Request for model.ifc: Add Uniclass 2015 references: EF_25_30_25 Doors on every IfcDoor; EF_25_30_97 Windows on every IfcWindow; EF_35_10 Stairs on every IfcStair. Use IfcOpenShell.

First a look at what the model holds.

```python
import ifcopenshell

model = ifcopenshell.open("model.ifc")
print(model.schema)
print("classifications:", [c.Name for c in model.by_type("IfcClassification")])
for ifc_class in ("IfcDoor", "IfcRoof", "IfcStair", "IfcWall", "IfcWindow"):
    print(ifc_class, len(model.by_type(ifc_class)))
```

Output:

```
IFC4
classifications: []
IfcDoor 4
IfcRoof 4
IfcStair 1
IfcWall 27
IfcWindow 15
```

```python
import ifcopenshell
import ifcopenshell.api.classification

model = ifcopenshell.open("model.ifc")

system = ifcopenshell.api.classification.add_classification(model, classification="Uniclass 2015")

codes = {
    "IfcDoor": ("EF_25_30_25", "Doors"),
    "IfcWindow": ("EF_25_30_97", "Windows"),
    "IfcStair": ("EF_35_10", "Stairs"),
}
for ifc_class, (code, name) in codes.items():
    products = model.by_type(ifc_class)
    ifcopenshell.api.classification.add_reference(
        model, products=products, classification=system, identification=code, name=name
    )
    print(code, len(products))

model.write("model_edited.ifc")
```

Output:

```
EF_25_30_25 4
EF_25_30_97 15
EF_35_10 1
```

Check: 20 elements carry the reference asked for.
